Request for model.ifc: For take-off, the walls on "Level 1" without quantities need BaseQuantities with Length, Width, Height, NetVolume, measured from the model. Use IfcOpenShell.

First a look at what the model holds.

```python
import ifcopenshell
import ifcopenshell.util.element
import ifcopenshell.util.unit

model = ifcopenshell.open("model.ifc")
print(model.schema)
for unit_type in ("LENGTHUNIT", "AREAUNIT", "VOLUMEUNIT"):
    print(unit_type, ifcopenshell.util.unit.calculate_unit_scale(model, unit_type))
storey = next(s for s in model.by_type("IfcBuildingStorey") if s.Name == "Level 1")
walls = [e for e in ifcopenshell.util.element.get_decomposition(storey) if e.is_a("IfcWall")]
for e in sorted(walls, key=lambda e: e.id()):
    print(e.id(), e.is_a(), e.Name, list(ifcopenshell.util.element.get_psets(e, qtos_only=True)), sep=" | ")
```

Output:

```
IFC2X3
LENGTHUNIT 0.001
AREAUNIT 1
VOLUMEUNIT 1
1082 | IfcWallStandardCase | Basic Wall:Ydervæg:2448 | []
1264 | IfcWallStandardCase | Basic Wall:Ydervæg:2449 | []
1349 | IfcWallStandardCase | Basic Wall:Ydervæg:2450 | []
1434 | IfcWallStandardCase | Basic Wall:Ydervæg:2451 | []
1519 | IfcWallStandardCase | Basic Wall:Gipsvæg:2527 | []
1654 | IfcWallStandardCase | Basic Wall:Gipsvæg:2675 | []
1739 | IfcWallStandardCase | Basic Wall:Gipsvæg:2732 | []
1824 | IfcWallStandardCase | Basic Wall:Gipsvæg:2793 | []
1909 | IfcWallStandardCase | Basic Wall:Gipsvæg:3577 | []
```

```python
import ifcopenshell
import ifcopenshell.api.pset
import ifcopenshell.geom
import ifcopenshell.util.element
import ifcopenshell.util.shape
import ifcopenshell.util.unit

model = ifcopenshell.open("model.ifc")
unit_scale = ifcopenshell.util.unit.calculate_unit_scale(model)
volume_scale = ifcopenshell.util.unit.calculate_unit_scale(model, "VOLUMEUNIT")
settings = ifcopenshell.geom.settings()

storey = next(s for s in model.by_type("IfcBuildingStorey") if s.Name == "Level 1")
walls = [e for e in ifcopenshell.util.element.get_decomposition(storey) if e.is_a("IfcWall")]

for e in sorted(walls, key=lambda e: e.id()):
    if ifcopenshell.util.element.get_psets(e, qtos_only=True, should_inherit=False):
        continue
    # Geometry comes back in metres, in the element's own axes.
    shape = ifcopenshell.geom.create_shape(settings, e)
    values = {
        "Length": ifcopenshell.util.shape.get_x(shape.geometry) / unit_scale,
        "Width": ifcopenshell.util.shape.get_y(shape.geometry) / unit_scale,
        "Height": ifcopenshell.util.shape.get_z(shape.geometry) / unit_scale,
        "NetVolume": ifcopenshell.util.shape.get_volume(shape.geometry) / volume_scale,
    }
    qto = ifcopenshell.api.pset.add_qto(model, product=e, name="BaseQuantities")
    ifcopenshell.api.pset.edit_qto(model, qto=qto, properties=values)
    print(e.id(), {k: round(v, 3) for k, v in values.items()})

model.write("model_updated.ifc")
```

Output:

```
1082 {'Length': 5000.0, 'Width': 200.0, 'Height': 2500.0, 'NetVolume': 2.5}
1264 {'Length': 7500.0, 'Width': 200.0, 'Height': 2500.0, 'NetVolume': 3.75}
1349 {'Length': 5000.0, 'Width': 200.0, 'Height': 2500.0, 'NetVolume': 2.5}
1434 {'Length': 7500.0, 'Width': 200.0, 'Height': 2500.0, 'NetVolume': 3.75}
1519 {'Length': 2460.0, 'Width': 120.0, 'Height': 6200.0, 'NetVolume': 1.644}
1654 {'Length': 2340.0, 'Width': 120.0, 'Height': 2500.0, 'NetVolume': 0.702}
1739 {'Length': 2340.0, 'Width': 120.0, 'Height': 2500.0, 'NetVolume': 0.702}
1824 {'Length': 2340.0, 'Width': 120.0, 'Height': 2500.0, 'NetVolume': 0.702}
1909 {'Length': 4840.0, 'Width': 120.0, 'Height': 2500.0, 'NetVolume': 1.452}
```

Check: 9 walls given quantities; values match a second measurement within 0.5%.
